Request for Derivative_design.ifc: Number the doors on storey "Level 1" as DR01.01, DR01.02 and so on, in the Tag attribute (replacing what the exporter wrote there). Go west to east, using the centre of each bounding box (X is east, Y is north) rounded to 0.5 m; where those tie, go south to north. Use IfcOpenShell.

First a look at what the model holds.

```python
import ifcopenshell
import ifcopenshell.util.element
import ifcopenshell.util.placement

model = ifcopenshell.open("Derivative_design.ifc")
print(model.schema)
storey = next(s for s in model.by_type("IfcBuildingStorey") if s.Name == "Level 1")
doors = [e for e in ifcopenshell.util.element.get_decomposition(storey) if e.is_a("IfcDoor")]
for e in sorted(doors, key=lambda e: e.id()):
    origin = ifcopenshell.util.placement.get_local_placement(e.ObjectPlacement)[:3, 3]
    print(e.id(), e.Tag, e.Name, origin.round(2) + 0.0, sep=" | ")
```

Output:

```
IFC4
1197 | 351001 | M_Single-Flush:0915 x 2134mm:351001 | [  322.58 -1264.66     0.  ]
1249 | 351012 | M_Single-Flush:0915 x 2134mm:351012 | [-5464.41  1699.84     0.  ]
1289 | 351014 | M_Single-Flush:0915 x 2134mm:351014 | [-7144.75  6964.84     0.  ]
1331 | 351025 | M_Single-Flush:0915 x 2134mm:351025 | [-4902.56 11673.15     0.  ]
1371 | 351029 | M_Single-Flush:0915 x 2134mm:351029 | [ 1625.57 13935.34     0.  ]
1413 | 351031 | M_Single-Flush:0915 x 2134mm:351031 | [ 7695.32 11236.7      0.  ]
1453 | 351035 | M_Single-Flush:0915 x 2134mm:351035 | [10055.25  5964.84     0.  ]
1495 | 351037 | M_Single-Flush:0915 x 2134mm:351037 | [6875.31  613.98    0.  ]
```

```python
import ifcopenshell
import ifcopenshell.geom
import ifcopenshell.util.element
import ifcopenshell.util.shape

model = ifcopenshell.open("Derivative_design.ifc")
settings = ifcopenshell.geom.settings()
settings.set("use-world-coords", True)


def centre(element):
    shape = ifcopenshell.geom.create_shape(settings, element)
    return ifcopenshell.util.shape.get_bbox_centroid(shape.geometry)


storey = next(s for s in model.by_type("IfcBuildingStorey") if s.Name == "Level 1")
doors = [e for e in ifcopenshell.util.element.get_decomposition(storey) if e.is_a("IfcDoor")]

# Insertion points can sit at a corner or the storey origin, so sort by the geometry (in metres).
centres = {e: centre(e) for e in doors}
doors.sort(key=lambda e: (round(centres[e][0] / 0.5), centres[e][1]))

for i, e in enumerate(doors, start=1):
    number = f"DR01.{i:02d}"
    e.Tag = number
    print(e.id(), number)

model.write("Derivative_design_v2.ifc")
```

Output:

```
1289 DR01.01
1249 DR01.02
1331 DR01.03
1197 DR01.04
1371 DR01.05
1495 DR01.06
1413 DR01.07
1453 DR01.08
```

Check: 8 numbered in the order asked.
